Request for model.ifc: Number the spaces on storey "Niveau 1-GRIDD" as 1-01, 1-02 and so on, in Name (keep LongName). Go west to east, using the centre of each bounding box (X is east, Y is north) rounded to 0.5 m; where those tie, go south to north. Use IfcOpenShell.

First a look at what the model holds.

```python
import ifcopenshell
import ifcopenshell.util.element
import ifcopenshell.util.placement

model = ifcopenshell.open("model.ifc")
print(model.schema)
storey = next(s for s in model.by_type("IfcBuildingStorey") if s.Name == "Niveau 1-GRIDD")
spaces = [e for e in ifcopenshell.util.element.get_decomposition(storey) if e.is_a("IfcSpace")]
for e in sorted(spaces, key=lambda e: e.id()):
    origin = ifcopenshell.util.placement.get_local_placement(e.ObjectPlacement)[:3, 3]
    print(e.id(), e.Name, e.LongName, origin.round(2) + 0.0, sep=" | ")
```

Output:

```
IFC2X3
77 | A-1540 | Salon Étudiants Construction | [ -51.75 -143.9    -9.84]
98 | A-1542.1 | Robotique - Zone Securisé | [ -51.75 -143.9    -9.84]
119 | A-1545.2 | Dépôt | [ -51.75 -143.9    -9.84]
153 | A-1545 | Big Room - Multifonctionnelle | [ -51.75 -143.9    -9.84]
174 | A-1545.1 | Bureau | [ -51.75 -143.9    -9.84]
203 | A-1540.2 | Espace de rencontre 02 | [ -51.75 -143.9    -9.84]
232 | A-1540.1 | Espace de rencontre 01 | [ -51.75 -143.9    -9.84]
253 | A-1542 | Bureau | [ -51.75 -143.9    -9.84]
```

```python
import ifcopenshell
import ifcopenshell.geom
import ifcopenshell.util.element
import ifcopenshell.util.shape

model = ifcopenshell.open("model.ifc")
settings = ifcopenshell.geom.settings()
settings.set("use-world-coords", True)


def centre(element):
    shape = ifcopenshell.geom.create_shape(settings, element)
    return ifcopenshell.util.shape.get_bbox_centroid(shape.geometry)


storey = next(s for s in model.by_type("IfcBuildingStorey") if s.Name == "Niveau 1-GRIDD")
spaces = [e for e in ifcopenshell.util.element.get_decomposition(storey) if e.is_a("IfcSpace")]

# Insertion points can sit at a corner or the storey origin, so sort by the geometry (in metres).
centres = {e: centre(e) for e in spaces}
spaces.sort(key=lambda e: (round(centres[e][0] / 0.5), centres[e][1]))

for i, e in enumerate(spaces, start=1):
    number = f"1-{i:02d}"
    e.Name = number
    print(e.id(), number)

model.write("model_edited.ifc")
```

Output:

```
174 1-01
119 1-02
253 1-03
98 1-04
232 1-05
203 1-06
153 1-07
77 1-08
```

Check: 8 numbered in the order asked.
